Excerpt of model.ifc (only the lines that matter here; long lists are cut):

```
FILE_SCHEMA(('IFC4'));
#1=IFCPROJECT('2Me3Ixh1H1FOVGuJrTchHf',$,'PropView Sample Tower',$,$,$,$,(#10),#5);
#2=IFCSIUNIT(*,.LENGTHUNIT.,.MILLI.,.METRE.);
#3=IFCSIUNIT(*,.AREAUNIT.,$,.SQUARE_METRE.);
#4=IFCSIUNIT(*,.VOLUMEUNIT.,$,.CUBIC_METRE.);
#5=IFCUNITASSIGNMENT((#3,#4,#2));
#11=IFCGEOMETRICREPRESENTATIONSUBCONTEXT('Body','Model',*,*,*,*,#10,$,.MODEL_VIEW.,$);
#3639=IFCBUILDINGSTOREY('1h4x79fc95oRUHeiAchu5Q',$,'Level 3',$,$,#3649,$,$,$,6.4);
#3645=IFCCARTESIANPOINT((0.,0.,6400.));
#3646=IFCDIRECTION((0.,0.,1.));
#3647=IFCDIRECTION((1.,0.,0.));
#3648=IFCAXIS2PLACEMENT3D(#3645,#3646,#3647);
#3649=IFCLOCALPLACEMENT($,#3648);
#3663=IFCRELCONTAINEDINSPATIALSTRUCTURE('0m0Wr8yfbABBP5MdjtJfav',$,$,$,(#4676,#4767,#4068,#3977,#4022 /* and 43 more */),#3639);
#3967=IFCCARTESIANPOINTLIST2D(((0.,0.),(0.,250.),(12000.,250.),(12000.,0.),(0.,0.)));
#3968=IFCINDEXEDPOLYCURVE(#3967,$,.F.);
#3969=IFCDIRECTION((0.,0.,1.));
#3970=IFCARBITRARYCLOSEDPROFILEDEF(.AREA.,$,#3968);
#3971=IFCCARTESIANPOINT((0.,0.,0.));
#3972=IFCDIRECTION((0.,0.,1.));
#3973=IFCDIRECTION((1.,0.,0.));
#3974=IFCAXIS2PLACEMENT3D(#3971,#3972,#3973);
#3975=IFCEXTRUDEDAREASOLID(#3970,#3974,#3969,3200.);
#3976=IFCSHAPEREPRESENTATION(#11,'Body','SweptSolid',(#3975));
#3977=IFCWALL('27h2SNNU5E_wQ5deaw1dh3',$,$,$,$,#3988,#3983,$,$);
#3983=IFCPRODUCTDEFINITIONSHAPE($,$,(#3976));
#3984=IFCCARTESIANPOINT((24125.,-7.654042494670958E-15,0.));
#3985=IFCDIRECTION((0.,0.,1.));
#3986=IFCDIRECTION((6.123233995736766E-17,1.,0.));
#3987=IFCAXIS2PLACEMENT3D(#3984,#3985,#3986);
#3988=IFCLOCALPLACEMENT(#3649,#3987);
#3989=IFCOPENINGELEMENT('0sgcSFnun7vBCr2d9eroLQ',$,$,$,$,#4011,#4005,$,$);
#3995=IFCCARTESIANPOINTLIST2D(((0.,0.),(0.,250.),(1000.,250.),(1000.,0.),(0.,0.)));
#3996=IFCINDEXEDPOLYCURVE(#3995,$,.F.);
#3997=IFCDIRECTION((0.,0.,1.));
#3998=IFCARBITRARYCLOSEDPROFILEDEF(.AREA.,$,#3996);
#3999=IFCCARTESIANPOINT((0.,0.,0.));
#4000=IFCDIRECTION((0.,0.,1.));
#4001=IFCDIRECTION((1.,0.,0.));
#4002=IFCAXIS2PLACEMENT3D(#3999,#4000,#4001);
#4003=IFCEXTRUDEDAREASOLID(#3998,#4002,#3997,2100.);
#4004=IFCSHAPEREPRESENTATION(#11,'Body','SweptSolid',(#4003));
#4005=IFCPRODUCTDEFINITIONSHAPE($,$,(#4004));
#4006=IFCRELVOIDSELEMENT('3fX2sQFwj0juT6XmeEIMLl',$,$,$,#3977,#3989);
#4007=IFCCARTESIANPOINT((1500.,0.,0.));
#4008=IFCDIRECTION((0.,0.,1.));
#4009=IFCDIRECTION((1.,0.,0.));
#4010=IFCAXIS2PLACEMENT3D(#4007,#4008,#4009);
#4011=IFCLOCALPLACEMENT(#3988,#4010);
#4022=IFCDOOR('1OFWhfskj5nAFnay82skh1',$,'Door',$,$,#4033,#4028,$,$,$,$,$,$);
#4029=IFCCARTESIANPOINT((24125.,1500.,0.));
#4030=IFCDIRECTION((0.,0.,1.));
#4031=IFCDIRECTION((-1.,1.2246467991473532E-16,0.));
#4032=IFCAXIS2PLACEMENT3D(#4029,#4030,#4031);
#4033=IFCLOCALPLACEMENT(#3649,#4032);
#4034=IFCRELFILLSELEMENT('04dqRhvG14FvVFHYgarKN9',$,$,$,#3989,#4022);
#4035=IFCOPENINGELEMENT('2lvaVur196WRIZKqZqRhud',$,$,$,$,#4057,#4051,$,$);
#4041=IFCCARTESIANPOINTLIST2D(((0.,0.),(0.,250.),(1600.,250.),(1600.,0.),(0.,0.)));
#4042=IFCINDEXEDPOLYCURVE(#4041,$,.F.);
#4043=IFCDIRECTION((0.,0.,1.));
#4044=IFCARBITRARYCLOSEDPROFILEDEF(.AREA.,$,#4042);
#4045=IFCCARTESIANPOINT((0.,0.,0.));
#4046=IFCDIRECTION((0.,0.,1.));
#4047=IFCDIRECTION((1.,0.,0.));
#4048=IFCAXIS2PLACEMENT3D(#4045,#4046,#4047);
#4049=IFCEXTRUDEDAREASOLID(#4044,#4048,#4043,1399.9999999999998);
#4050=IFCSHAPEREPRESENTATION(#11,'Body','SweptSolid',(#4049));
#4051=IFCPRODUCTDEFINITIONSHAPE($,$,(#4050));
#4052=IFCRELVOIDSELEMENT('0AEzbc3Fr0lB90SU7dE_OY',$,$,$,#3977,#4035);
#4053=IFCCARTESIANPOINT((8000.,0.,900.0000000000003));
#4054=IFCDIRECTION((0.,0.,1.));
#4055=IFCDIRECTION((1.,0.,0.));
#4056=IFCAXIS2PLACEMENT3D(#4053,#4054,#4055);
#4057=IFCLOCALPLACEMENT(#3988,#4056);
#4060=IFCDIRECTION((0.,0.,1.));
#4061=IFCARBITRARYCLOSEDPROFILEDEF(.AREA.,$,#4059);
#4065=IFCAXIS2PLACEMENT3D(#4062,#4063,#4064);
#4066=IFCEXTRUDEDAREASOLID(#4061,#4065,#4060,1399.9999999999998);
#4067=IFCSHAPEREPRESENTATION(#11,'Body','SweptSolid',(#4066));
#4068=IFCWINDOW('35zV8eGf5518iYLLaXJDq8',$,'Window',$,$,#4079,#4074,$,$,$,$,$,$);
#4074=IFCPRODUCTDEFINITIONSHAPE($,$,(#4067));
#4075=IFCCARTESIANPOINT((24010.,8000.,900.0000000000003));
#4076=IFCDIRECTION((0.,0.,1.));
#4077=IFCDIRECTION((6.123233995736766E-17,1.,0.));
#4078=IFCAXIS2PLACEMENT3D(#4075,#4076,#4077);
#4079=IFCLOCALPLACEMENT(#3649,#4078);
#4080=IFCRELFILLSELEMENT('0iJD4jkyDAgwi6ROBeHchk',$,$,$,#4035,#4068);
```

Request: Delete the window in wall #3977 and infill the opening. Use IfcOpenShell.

```python
import ifcopenshell
import ifcopenshell.api.feature
import ifcopenshell.api.root
import ifcopenshell.geom
import ifcopenshell.util.shape

model = ifcopenshell.open("model.ifc")
settings = ifcopenshell.geom.settings()


def volume(element):
    """Net volume in cubic metres, openings subtracted."""
    shape = ifcopenshell.geom.create_shape(settings, element)
    return ifcopenshell.util.shape.get_volume(shape.geometry)


window = model.by_id(4068)
opening = window.FillsVoids[0].RelatingOpeningElement
wall = opening.VoidsElements[0].RelatingBuildingElement
before = volume(wall)

ifcopenshell.api.root.remove_product(model, product=window)
ifcopenshell.api.feature.remove_feature(model, feature=opening)

after = volume(wall)

print(f"wall volume {before:.3f} -> {after:.3f} m3")

model.write("model_rev.ifc")
```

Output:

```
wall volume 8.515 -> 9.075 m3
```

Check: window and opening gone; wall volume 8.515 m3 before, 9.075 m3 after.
